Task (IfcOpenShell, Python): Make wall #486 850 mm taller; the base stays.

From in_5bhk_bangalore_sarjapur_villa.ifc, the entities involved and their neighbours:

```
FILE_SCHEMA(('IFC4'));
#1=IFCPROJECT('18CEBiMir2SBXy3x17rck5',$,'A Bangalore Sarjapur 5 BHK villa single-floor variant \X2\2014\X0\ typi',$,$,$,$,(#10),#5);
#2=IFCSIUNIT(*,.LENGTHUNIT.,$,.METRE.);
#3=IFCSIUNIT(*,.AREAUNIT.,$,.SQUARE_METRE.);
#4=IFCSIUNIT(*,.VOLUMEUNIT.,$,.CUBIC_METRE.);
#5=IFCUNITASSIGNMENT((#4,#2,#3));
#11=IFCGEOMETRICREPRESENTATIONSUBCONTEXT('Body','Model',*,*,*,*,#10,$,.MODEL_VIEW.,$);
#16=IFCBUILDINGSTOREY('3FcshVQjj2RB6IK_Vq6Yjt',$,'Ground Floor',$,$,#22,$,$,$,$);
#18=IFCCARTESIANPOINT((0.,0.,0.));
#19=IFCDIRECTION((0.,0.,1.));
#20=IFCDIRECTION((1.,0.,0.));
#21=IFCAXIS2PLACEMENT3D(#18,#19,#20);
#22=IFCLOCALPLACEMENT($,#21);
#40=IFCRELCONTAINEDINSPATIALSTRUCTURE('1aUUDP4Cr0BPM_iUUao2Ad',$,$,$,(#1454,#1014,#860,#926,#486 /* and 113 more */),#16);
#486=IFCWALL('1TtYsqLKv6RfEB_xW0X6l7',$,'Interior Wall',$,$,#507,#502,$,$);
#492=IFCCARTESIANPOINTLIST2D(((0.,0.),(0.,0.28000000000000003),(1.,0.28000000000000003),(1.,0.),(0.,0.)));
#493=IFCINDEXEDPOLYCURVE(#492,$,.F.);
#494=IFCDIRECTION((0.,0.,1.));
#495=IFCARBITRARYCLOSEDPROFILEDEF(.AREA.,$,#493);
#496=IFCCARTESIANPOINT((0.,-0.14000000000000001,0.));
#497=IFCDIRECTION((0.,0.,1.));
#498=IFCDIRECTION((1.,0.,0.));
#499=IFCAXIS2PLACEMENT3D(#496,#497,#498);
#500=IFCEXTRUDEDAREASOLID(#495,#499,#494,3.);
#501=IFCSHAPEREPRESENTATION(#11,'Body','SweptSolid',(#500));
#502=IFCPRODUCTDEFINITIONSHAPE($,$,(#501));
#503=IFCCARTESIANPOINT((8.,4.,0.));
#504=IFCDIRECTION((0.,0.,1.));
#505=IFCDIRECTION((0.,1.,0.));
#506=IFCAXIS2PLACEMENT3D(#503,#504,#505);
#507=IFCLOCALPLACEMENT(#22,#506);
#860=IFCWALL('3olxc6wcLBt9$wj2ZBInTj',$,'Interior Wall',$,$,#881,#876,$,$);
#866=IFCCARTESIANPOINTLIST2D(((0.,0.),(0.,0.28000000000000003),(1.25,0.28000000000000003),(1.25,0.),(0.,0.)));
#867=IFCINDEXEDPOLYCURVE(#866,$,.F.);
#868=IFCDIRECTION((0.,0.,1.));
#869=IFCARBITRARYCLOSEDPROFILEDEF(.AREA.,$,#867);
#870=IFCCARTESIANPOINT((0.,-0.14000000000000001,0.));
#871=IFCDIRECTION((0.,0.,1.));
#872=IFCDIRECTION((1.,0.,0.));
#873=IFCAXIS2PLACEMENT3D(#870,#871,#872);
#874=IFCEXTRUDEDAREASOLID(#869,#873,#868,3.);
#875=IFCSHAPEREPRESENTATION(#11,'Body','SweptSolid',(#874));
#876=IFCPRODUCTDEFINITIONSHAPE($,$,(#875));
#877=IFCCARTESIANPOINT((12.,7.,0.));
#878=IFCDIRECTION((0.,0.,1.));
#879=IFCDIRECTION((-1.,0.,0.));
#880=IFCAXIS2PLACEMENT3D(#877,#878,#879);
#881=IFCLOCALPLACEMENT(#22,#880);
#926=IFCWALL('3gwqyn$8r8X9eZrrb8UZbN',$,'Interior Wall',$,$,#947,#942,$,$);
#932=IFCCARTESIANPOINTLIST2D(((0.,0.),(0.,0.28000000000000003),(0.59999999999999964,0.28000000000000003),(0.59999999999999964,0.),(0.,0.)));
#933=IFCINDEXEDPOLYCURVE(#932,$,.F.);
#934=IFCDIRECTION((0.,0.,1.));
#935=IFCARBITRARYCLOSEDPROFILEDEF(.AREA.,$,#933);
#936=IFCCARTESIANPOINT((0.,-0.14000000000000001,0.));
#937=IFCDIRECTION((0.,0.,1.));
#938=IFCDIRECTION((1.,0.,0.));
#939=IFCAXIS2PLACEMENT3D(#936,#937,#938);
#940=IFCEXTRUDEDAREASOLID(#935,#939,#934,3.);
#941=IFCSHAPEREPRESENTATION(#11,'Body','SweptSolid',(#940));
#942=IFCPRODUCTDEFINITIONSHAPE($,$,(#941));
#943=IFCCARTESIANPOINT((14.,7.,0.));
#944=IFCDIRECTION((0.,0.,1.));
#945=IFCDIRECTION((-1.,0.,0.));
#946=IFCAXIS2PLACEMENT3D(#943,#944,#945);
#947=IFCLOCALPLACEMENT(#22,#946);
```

```python
import ifcopenshell
import ifcopenshell.geom
import ifcopenshell.util.representation
import ifcopenshell.util.shape
import ifcopenshell.util.unit

model = ifcopenshell.open("in_5bhk_bangalore_sarjapur_villa.ifc")
unit_scale = ifcopenshell.util.unit.calculate_unit_scale(model)
settings = ifcopenshell.geom.settings()


def volume(element):
    """Net volume in cubic metres, openings subtracted."""
    shape = ifcopenshell.geom.create_shape(settings, element)
    return ifcopenshell.util.shape.get_volume(shape.geometry)


wall = model.by_guid("1TtYsqLKv6RfEB_xW0X6l7")
before = volume(wall)

body = ifcopenshell.util.representation.get_representation(wall, "Model", "Body")
solid = body.Items[0]
old_height = solid.Depth
solid.Depth += 0.85 / unit_scale
after = volume(wall)

print(f"height {old_height:g} -> {solid.Depth:g}, volume {before:.3f} -> {after:.3f} m3")

model.write("in_5bhk_bangalore_sarjapur_villa_edited.ifc")
```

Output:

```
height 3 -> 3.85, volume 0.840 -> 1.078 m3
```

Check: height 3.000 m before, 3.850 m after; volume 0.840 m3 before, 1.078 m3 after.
